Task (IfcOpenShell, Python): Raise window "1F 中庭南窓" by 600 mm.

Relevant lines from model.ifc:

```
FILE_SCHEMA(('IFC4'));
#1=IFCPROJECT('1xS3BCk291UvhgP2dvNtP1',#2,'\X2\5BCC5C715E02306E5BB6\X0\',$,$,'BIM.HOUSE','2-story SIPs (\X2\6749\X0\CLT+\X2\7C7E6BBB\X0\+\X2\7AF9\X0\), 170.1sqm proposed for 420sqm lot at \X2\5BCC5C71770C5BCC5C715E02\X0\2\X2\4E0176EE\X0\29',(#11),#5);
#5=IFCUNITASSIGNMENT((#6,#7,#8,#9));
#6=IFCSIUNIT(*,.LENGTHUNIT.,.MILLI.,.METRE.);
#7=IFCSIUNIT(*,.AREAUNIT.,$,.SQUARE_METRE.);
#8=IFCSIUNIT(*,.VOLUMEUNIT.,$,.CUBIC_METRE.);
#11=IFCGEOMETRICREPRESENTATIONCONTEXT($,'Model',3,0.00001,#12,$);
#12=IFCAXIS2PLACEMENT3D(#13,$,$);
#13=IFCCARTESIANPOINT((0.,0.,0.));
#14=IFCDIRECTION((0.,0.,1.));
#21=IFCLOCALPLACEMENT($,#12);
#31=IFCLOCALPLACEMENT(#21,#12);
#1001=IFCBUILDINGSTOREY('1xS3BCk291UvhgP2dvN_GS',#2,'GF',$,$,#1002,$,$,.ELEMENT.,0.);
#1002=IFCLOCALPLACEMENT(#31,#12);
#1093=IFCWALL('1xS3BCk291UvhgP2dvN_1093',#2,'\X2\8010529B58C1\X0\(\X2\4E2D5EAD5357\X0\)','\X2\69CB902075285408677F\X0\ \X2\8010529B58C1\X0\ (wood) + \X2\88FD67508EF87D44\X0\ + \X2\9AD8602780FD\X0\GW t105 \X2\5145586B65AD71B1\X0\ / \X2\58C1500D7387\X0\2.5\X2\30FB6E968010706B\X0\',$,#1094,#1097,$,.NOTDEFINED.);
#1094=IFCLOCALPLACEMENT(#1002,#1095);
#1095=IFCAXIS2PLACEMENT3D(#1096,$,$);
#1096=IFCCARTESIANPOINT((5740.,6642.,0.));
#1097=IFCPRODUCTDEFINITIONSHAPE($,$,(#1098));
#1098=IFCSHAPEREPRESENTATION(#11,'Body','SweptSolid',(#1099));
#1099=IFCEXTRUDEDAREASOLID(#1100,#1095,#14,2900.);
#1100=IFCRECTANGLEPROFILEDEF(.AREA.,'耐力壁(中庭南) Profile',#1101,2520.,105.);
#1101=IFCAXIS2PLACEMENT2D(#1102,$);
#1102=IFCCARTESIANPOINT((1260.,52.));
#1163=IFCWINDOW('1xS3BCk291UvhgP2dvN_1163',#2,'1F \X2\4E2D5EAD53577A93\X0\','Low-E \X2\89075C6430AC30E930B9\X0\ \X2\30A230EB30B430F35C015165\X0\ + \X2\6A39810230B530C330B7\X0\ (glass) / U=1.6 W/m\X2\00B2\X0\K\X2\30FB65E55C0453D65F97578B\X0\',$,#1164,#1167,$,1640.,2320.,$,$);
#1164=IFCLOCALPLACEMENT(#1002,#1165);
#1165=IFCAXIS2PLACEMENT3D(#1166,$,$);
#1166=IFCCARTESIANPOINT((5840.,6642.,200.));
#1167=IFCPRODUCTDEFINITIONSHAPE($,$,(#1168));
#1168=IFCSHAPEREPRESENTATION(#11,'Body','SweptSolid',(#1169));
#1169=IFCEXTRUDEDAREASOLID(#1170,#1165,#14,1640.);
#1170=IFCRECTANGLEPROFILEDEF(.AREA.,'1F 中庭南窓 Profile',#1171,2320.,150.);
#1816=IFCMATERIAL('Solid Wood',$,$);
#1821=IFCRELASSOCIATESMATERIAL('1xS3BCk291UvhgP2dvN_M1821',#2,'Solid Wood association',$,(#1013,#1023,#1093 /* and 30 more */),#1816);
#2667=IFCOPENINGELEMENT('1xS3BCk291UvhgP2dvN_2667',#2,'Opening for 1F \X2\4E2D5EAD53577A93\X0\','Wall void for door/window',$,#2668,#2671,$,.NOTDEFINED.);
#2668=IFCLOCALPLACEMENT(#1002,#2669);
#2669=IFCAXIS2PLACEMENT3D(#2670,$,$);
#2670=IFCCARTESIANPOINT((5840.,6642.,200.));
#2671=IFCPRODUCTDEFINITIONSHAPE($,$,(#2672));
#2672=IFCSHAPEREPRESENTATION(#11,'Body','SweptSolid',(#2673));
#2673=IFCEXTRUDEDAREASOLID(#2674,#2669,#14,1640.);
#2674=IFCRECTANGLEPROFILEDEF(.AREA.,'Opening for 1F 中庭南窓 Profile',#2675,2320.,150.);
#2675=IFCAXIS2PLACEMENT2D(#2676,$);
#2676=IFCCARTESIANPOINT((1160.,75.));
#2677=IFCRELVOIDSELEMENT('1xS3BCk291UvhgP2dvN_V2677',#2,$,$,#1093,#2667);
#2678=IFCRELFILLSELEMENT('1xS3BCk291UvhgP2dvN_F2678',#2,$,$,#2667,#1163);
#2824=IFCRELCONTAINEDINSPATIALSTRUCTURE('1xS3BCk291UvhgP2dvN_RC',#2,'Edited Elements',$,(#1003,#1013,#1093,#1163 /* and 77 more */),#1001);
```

```python
import numpy as np
import ifcopenshell
import ifcopenshell.api.geometry
import ifcopenshell.util.placement
import ifcopenshell.util.unit

model = ifcopenshell.open("model.ifc")
unit_scale = ifcopenshell.util.unit.calculate_unit_scale(model)

window = model.by_guid("1xS3BCk291UvhgP2dvN_1163")
opening = window.FillsVoids[0].RelatingOpeningElement
dz = 0.6 / unit_scale

shift = np.array([0.0, 0.0, dz])
# The window is not placed relative to its opening, so move both.
for product in (opening, window):
    matrix = ifcopenshell.util.placement.get_local_placement(product.ObjectPlacement)
    matrix[:3, 3] += shift
    ifcopenshell.api.geometry.edit_object_placement(model, product=product, matrix=matrix, is_si=False)

print(f"moved by {dz * unit_scale:+.3f} m")

model.write("model_v2.ifc")
```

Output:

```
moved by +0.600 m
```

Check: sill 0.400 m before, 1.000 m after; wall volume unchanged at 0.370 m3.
